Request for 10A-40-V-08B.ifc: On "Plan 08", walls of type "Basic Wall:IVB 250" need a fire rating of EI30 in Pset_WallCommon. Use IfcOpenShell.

First a look at what the model holds.

```python
import ifcopenshell
import ifcopenshell.util.element

model = ifcopenshell.open("10A-40-V-08B.ifc")
print(model.schema)
storey = next(s for s in model.by_type("IfcBuildingStorey") if s.Name == "Plan 08")
walls = [e for e in ifcopenshell.util.element.get_decomposition(storey) if e.is_a("IfcWall")]
seen = {}
for e in walls:
    element_type = ifcopenshell.util.element.get_type(e)
    key = (element_type.Name if element_type != e and element_type else None, ifcopenshell.util.element.get_pset(e, "Pset_WallCommon", "FireRating"))
    seen[key] = seen.get(key, 0) + 1
for (name, value), count in sorted(seen.items(), key=str):
    print(count, "x", name, "|", value)
```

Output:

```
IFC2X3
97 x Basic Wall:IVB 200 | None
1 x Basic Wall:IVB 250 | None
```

```python
import ifcopenshell
import ifcopenshell.api.pset
import ifcopenshell.util.element

model = ifcopenshell.open("10A-40-V-08B.ifc")

storey = next(s for s in model.by_type("IfcBuildingStorey") if s.Name == "Plan 08")
walls = [e for e in ifcopenshell.util.element.get_decomposition(storey) if e.is_a("IfcWall")]

count = 0
for e in walls:
    element_type = ifcopenshell.util.element.get_type(e)
    if element_type in (None, e) or element_type.Name != "Basic Wall:IVB 250":
        continue
    found = ifcopenshell.util.element.get_pset(e, "Pset_WallCommon", should_inherit=False)
    if found:
        pset = model.by_id(found["id"])
        if len(ifcopenshell.util.element.get_elements_by_pset(pset)) > 1:
            pset = ifcopenshell.api.pset.unshare_pset(model, products=[e], pset=pset)[0]
    else:
        pset = ifcopenshell.api.pset.add_pset(model, product=e, name="Pset_WallCommon")
    ifcopenshell.api.pset.edit_pset(model, pset=pset, properties={"FireRating": "EI30"})
    count += 1

print(count, "walls updated")

model.write("10A-40-V-08B_rev.ifc")
```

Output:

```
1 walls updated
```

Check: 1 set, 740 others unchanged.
